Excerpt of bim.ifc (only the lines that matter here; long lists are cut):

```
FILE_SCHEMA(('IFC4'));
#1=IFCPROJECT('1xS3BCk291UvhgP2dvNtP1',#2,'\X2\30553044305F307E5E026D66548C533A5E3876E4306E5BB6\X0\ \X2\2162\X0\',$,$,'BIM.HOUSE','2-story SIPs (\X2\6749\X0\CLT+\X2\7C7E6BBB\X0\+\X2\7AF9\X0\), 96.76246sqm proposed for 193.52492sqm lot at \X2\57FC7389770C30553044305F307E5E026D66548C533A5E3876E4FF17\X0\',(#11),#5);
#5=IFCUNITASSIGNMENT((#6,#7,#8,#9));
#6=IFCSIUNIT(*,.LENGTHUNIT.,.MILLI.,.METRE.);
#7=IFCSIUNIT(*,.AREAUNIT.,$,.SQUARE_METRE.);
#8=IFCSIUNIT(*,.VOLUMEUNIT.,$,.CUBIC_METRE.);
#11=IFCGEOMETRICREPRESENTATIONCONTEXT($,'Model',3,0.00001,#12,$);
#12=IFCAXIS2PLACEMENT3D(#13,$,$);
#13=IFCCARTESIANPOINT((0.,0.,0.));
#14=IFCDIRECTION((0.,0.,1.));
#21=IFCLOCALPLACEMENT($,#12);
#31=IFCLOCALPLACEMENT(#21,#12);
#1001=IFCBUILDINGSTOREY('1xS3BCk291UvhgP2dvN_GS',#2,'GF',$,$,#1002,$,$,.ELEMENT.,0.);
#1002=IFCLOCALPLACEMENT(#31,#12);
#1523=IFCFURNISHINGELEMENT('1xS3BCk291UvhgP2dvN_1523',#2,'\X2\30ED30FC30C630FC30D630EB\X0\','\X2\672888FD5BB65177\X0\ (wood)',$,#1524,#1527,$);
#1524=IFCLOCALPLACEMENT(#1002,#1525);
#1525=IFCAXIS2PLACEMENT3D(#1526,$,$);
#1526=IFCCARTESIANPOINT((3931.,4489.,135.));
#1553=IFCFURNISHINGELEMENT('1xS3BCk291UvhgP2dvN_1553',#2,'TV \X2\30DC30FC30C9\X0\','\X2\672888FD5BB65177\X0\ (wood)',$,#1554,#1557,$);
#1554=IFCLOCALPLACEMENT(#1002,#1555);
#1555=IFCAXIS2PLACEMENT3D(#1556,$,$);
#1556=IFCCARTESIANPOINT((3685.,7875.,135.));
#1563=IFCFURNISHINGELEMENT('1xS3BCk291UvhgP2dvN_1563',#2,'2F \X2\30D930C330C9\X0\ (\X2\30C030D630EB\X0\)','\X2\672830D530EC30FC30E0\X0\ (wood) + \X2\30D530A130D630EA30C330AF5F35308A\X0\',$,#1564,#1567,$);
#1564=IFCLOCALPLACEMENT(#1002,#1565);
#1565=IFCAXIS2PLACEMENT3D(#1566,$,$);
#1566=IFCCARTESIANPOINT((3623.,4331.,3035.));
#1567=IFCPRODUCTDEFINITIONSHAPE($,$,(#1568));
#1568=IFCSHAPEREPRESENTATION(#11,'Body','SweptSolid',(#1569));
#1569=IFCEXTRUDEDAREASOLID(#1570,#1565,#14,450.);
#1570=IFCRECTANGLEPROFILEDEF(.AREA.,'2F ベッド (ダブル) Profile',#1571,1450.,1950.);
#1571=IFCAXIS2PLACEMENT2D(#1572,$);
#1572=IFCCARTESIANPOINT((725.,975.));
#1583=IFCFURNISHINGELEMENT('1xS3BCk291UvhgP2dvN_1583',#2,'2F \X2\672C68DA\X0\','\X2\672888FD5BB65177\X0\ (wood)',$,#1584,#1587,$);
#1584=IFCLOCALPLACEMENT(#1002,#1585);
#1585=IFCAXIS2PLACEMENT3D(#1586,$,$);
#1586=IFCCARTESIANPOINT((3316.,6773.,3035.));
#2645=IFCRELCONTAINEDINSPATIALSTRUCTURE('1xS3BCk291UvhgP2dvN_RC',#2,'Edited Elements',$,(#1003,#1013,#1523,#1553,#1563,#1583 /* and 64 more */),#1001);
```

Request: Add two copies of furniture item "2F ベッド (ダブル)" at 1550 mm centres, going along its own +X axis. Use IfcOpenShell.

```python
import ifcopenshell
import ifcopenshell.api.geometry
import ifcopenshell.api.root
import ifcopenshell.util.element
import ifcopenshell.util.placement

model = ifcopenshell.open("bim.ifc")


def reuse_history(source, copy):
    """copy_class also copies each property set's owner history, people and application; keep the originals."""
    for rel in copy.IsDefinedBy:
        if rel.is_a("IfcRelDefinesByProperties") and (history := rel.RelatingPropertyDefinition.OwnerHistory):
            rel.RelatingPropertyDefinition.OwnerHistory = source.OwnerHistory
            ifcopenshell.util.element.remove_deep2(model, history)


source = model.by_id(1563)
base = ifcopenshell.util.placement.get_local_placement(source.ObjectPlacement)
step = base[:3, 0] * 1550.0

for i in range(1, 3):
    copy = ifcopenshell.api.root.copy_class(model, product=source)
    copy.Representation = ifcopenshell.util.element.copy_deep(
        model, source.Representation, exclude=["IfcGeometricRepresentationContext", "IfcRepresentationMap"]
    )
    reuse_history(source, copy)
    matrix = base.copy()
    matrix[:3, 3] += i * step
    print("added at", matrix[:3, 3].round(3) + 0.0)
    ifcopenshell.api.geometry.edit_object_placement(model, product=copy, matrix=matrix, is_si=False)

model.write("bim_updated.ifc")
```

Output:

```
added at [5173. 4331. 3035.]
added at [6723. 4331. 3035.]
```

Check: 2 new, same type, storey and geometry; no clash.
